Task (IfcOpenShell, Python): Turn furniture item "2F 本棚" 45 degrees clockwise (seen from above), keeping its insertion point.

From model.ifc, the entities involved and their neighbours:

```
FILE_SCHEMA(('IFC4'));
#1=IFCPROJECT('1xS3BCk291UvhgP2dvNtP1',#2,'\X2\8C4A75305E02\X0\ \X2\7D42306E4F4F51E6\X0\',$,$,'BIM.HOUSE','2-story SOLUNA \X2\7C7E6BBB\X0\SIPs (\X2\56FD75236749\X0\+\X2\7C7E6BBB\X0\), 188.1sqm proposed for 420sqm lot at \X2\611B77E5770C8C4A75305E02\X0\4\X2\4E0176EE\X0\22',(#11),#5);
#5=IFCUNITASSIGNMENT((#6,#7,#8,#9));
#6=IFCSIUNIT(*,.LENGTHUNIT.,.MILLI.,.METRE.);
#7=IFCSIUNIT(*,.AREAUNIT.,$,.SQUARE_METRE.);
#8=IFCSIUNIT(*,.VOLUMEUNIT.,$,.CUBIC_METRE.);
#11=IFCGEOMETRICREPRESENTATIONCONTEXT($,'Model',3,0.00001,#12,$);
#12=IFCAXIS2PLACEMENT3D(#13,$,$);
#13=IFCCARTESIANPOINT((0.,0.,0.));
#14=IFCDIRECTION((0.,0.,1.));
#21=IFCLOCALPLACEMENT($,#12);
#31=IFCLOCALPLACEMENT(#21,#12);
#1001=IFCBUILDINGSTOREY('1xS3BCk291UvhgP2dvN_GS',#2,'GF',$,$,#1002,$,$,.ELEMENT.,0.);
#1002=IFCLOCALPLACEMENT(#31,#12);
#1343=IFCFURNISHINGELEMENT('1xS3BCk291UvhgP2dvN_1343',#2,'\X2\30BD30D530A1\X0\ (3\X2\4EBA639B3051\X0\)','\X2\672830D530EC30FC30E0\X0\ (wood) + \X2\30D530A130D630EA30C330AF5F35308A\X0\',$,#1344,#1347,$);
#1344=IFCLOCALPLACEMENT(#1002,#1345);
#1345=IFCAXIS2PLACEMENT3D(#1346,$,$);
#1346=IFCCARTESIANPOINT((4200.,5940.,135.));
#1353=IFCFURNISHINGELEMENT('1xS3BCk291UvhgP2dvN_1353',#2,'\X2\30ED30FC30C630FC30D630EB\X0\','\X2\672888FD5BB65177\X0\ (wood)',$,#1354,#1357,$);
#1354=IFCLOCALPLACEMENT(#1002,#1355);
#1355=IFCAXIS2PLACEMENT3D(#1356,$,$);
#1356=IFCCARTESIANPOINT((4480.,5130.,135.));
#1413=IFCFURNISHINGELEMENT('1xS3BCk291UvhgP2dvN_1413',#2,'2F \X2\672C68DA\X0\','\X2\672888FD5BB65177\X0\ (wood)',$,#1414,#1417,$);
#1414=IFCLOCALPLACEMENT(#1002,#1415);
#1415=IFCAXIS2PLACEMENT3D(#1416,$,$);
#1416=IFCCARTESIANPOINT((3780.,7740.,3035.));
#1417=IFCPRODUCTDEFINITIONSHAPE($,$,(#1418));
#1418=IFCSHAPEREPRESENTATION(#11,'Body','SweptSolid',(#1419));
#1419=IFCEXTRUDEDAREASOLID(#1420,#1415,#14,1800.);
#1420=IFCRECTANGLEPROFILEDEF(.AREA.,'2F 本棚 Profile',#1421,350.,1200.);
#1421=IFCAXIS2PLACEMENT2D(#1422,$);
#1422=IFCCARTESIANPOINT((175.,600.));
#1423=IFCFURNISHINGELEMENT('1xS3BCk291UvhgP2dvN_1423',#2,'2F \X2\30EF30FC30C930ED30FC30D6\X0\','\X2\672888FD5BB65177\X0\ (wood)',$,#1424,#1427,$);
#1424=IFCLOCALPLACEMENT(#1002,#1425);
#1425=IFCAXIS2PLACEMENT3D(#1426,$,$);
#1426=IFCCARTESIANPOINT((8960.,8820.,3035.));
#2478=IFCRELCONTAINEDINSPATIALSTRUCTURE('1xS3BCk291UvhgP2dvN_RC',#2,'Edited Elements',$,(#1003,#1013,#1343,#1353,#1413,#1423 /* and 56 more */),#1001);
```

```python
import ifcopenshell
import ifcopenshell.api.geometry
import ifcopenshell.util.placement

model = ifcopenshell.open("model.ifc")

item = model.by_guid("1xS3BCk291UvhgP2dvN_1413")
matrix = ifcopenshell.util.placement.get_local_placement(item.ObjectPlacement)
matrix = matrix @ ifcopenshell.util.placement.rotation(-45, "Z")
ifcopenshell.api.geometry.edit_object_placement(model, product=item, matrix=matrix, is_si=False)

print(ifcopenshell.util.placement.get_local_placement(item.ObjectPlacement).round(3) + 0.0)

model.write("model-out.ifc")
```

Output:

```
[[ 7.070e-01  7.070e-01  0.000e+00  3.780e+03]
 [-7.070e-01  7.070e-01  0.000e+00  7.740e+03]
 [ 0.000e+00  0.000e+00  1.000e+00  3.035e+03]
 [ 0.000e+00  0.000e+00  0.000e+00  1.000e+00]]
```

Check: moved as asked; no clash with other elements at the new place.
